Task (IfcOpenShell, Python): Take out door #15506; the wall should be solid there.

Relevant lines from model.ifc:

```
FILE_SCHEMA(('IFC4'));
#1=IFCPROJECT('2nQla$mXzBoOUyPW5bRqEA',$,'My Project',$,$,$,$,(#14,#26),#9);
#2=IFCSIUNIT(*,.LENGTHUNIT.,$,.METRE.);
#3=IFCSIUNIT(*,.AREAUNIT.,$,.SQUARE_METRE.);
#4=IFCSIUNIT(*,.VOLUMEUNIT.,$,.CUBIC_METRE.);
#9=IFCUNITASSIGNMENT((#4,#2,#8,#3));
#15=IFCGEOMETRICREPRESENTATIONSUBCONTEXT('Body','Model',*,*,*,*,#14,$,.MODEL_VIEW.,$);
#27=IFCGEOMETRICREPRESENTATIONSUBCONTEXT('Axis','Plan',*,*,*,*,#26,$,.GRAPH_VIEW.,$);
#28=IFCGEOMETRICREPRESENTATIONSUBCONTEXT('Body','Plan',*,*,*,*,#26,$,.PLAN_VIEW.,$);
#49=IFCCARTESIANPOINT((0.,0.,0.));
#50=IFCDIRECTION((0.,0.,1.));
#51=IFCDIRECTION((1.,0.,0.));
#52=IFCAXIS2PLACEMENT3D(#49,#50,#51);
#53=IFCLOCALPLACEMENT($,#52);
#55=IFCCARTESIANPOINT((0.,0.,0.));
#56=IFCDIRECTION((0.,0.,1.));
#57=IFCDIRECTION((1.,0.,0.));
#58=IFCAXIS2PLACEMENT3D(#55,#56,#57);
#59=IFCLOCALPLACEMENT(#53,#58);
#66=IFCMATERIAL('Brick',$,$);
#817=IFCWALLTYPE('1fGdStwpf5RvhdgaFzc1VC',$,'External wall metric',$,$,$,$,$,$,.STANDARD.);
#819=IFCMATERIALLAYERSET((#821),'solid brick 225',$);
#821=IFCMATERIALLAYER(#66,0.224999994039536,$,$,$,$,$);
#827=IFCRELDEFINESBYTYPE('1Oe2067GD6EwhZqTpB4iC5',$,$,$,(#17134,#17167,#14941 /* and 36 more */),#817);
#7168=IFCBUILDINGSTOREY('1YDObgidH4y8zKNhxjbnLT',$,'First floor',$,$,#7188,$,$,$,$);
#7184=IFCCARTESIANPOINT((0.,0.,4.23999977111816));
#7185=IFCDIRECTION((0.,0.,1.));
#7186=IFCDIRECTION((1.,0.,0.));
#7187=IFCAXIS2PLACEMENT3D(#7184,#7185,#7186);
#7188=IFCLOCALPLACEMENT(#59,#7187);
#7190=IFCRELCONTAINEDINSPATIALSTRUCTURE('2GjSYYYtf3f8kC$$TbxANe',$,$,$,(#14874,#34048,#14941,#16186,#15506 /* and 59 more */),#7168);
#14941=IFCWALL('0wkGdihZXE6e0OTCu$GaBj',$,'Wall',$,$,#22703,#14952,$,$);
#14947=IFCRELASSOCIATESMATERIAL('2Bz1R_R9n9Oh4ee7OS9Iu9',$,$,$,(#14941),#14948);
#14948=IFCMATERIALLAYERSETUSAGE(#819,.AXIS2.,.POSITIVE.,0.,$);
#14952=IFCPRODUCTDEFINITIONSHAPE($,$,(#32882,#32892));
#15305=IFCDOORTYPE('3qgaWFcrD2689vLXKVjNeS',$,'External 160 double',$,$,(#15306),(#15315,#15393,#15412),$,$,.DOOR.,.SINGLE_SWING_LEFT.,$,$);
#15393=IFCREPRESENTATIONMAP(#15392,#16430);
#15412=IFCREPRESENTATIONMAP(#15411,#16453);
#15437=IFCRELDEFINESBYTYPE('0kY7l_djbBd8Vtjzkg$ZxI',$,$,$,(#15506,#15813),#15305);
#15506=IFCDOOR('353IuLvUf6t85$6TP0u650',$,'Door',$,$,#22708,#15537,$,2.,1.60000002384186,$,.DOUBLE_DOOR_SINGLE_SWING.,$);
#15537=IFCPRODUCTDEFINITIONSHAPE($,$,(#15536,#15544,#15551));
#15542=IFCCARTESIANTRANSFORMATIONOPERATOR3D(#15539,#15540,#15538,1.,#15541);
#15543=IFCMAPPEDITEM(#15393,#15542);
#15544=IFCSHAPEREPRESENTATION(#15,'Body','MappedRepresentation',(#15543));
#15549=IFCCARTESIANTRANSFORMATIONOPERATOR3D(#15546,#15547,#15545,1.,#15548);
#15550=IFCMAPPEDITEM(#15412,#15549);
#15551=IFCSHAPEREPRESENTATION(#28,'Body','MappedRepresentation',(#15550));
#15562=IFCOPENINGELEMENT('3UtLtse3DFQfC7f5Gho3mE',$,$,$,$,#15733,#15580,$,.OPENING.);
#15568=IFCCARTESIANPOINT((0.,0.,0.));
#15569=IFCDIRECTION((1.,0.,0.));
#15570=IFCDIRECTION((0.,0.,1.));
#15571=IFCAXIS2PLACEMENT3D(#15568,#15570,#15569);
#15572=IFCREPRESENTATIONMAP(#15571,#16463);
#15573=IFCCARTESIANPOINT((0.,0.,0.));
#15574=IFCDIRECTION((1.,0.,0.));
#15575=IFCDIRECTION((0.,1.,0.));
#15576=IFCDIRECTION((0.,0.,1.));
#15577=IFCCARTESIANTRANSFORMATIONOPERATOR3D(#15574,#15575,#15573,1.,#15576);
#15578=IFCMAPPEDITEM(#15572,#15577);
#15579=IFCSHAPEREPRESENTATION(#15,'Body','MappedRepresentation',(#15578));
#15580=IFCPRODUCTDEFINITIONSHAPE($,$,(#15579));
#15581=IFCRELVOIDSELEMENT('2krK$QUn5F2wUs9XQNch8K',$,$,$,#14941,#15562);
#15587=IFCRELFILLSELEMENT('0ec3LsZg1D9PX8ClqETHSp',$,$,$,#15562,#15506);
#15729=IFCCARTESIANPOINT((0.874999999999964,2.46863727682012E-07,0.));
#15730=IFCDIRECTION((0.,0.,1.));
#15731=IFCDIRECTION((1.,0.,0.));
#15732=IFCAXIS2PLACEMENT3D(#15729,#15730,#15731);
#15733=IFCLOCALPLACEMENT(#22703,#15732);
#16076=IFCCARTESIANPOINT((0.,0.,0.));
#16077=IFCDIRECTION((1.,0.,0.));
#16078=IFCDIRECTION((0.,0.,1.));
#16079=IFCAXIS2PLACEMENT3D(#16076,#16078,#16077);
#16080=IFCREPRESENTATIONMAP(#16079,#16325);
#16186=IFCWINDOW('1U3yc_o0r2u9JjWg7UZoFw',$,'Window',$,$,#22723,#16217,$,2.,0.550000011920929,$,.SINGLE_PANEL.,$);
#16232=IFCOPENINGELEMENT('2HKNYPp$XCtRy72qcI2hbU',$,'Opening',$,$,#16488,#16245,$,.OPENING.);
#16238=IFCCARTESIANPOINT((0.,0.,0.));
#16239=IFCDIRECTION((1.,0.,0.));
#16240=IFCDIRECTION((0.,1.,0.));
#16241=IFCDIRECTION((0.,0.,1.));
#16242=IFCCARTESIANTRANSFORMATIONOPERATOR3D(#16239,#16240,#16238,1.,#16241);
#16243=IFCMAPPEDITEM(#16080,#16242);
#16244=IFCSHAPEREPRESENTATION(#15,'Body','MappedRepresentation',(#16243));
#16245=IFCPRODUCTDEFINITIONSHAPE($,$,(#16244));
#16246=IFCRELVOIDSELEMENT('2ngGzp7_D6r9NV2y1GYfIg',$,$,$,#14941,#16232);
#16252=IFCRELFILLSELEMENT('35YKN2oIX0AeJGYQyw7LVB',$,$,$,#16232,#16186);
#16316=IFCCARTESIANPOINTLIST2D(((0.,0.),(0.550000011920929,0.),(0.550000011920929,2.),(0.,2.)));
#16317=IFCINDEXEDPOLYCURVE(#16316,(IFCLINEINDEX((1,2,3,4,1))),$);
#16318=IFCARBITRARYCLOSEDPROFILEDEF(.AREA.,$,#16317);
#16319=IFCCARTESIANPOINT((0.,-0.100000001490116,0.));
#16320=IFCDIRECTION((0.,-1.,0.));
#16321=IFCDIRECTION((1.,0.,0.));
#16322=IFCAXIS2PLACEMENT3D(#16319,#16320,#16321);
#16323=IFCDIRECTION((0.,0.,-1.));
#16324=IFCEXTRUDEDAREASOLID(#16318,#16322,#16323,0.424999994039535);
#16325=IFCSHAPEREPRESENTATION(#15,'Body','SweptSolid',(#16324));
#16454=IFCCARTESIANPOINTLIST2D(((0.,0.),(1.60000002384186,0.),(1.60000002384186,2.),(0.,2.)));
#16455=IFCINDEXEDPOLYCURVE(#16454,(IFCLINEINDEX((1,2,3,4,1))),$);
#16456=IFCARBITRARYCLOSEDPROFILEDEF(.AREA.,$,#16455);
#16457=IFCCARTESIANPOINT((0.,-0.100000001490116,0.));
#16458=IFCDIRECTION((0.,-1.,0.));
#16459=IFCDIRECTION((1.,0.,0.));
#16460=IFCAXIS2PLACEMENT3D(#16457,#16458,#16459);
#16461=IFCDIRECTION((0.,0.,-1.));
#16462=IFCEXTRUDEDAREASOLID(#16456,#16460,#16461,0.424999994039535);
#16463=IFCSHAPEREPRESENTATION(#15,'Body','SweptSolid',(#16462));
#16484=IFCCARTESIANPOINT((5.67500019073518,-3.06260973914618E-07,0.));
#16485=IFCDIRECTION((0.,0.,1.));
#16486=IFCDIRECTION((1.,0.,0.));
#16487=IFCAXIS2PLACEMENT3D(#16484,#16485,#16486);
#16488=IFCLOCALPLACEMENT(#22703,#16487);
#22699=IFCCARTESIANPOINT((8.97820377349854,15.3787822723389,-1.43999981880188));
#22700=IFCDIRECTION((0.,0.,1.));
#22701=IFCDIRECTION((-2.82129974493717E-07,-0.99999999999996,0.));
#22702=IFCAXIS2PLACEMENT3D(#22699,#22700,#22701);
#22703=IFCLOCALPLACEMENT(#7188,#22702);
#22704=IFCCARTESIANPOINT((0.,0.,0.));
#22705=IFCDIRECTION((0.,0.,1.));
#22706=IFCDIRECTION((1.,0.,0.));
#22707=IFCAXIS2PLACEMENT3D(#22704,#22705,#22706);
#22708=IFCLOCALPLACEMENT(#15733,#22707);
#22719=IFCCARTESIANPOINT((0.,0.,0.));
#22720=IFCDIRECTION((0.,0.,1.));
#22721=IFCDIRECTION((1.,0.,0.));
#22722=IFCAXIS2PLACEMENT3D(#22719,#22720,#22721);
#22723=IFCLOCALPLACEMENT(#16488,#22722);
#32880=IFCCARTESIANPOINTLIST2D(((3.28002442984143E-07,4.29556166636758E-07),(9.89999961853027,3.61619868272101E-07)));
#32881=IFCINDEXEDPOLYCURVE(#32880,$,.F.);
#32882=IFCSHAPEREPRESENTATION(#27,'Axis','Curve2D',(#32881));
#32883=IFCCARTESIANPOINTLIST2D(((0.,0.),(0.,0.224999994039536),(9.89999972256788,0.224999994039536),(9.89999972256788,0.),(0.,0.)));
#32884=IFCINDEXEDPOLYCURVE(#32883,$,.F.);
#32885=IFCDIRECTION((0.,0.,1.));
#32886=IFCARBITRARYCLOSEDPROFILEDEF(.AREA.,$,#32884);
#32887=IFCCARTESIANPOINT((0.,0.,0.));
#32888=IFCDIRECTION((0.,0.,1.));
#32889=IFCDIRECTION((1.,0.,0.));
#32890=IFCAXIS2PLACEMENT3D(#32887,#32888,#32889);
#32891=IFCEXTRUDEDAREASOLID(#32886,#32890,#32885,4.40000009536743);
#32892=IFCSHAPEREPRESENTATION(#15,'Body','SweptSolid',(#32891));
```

```python
import ifcopenshell
import ifcopenshell.api.feature
import ifcopenshell.api.root
import ifcopenshell.geom
import ifcopenshell.util.shape

model = ifcopenshell.open("model.ifc")
settings = ifcopenshell.geom.settings()


def volume(element):
    """Net volume in cubic metres, openings subtracted."""
    shape = ifcopenshell.geom.create_shape(settings, element)
    return ifcopenshell.util.shape.get_volume(shape.geometry)


door = model.by_guid("353IuLvUf6t85$6TP0u650")
opening = door.FillsVoids[0].RelatingOpeningElement
wall = opening.VoidsElements[0].RelatingBuildingElement
before = volume(wall)

ifcopenshell.api.root.remove_product(model, product=door)
ifcopenshell.api.feature.remove_feature(model, feature=opening)

after = volume(wall)

print(f"wall volume {before:.3f} -> {after:.3f} m3")

model.write("model_edited.ifc")
```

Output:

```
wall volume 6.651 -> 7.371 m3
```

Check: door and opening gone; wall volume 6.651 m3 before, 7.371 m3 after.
